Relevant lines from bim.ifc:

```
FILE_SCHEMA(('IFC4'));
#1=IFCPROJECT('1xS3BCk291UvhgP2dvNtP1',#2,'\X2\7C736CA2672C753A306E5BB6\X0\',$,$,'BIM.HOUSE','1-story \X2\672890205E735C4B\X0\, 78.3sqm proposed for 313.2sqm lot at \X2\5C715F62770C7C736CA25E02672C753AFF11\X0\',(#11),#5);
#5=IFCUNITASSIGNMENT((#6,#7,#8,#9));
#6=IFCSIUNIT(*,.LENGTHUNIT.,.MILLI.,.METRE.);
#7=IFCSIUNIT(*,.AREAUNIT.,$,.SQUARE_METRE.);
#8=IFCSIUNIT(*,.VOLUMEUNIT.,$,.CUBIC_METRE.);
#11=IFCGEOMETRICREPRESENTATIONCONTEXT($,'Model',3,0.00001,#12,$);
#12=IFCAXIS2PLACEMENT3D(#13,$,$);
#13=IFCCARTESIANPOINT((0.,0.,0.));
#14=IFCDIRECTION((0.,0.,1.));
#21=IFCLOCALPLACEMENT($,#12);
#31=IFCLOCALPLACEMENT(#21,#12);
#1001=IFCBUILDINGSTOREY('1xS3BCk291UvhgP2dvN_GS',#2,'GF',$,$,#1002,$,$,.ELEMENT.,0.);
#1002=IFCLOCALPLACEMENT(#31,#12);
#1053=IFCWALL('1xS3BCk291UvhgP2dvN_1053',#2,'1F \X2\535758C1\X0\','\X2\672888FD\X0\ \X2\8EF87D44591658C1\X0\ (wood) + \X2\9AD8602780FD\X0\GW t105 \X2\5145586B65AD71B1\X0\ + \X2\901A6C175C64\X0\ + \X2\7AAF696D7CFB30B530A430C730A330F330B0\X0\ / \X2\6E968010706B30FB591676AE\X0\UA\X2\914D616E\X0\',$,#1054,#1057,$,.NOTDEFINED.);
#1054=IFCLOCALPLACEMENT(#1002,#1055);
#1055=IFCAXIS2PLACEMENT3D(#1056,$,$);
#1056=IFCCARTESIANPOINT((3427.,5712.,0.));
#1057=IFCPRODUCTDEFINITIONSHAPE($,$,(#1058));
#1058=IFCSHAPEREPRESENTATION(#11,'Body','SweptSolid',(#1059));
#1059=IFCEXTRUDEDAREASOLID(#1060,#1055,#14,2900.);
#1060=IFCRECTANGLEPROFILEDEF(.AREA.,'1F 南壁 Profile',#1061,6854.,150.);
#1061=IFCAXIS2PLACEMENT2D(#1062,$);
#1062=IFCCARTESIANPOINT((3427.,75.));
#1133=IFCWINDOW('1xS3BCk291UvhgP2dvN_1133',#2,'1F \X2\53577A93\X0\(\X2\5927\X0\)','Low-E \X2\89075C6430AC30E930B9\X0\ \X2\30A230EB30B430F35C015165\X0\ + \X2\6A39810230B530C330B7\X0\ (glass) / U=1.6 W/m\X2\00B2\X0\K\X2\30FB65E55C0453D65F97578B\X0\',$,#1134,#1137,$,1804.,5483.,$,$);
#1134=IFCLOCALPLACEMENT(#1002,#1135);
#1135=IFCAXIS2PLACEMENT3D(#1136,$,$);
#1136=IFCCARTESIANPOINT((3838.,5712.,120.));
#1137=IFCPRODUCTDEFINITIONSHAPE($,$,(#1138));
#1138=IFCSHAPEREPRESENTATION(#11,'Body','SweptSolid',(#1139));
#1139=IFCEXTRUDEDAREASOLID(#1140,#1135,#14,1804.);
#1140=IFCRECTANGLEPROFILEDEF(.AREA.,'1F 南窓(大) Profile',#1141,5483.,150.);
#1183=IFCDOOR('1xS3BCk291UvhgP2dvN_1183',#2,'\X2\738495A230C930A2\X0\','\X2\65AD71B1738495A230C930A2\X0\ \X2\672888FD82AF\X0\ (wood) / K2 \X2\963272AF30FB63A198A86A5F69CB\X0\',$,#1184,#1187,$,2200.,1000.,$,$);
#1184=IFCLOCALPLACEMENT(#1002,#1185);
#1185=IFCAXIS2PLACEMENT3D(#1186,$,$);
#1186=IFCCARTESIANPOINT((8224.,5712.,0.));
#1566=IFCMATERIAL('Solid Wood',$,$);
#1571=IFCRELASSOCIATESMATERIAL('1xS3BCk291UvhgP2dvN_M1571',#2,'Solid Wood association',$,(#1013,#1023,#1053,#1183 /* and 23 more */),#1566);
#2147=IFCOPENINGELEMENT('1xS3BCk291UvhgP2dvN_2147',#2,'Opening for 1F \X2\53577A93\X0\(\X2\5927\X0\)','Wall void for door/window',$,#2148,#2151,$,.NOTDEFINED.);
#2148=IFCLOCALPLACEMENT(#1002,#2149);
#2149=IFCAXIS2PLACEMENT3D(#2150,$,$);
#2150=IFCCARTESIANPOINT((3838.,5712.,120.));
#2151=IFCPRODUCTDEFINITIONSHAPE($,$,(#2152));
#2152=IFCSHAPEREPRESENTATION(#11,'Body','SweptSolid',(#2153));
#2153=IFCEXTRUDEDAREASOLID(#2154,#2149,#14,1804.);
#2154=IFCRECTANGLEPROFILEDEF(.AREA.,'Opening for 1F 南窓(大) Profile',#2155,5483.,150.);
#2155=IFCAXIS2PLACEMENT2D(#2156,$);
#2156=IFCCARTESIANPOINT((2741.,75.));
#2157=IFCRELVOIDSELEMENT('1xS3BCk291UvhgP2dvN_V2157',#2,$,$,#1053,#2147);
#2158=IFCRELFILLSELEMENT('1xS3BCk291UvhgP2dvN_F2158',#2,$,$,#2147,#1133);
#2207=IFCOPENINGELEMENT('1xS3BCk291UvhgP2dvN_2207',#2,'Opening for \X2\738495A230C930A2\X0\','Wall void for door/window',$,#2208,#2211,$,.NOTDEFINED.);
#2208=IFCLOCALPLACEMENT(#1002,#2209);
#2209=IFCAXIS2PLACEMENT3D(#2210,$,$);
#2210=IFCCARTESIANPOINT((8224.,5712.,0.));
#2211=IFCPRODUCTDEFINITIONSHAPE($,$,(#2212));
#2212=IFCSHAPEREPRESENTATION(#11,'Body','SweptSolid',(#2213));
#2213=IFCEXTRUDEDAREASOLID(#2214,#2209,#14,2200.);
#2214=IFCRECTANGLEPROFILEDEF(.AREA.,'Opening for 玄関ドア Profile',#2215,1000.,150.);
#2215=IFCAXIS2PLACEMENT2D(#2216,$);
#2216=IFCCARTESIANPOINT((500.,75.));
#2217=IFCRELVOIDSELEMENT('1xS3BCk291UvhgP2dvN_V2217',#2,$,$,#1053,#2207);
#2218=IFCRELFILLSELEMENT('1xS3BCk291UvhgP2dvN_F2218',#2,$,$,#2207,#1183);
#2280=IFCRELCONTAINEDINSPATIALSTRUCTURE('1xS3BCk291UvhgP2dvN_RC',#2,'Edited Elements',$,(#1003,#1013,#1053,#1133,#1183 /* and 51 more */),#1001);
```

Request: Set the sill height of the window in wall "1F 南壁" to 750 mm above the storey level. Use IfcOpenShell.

```python
import numpy as np
import ifcopenshell
import ifcopenshell.api.geometry
import ifcopenshell.geom
import ifcopenshell.util.element
import ifcopenshell.util.placement
import ifcopenshell.util.shape
import ifcopenshell.util.unit

model = ifcopenshell.open("bim.ifc")
unit_scale = ifcopenshell.util.unit.calculate_unit_scale(model)

window = model.by_guid("1xS3BCk291UvhgP2dvN_1133")
opening = window.FillsVoids[0].RelatingOpeningElement
storey = ifcopenshell.util.element.get_container(window, ifc_class="IfcBuildingStorey")
level = ifcopenshell.util.placement.get_local_placement(storey.ObjectPlacement)[2, 3]

# The opening's origin need not be at the sill, so measure its lowest point.
shape = ifcopenshell.geom.create_shape(ifcopenshell.geom.settings(), opening)
bottom = ifcopenshell.util.shape.get_shape_bottom_elevation(shape, shape.geometry) / unit_scale
dz = level + 0.75 / unit_scale - bottom

shift = np.array([0.0, 0.0, dz])
# The window is not placed relative to its opening, so move both.
for product in (opening, window):
    matrix = ifcopenshell.util.placement.get_local_placement(product.ObjectPlacement)
    matrix[:3, 3] += shift
    ifcopenshell.api.geometry.edit_object_placement(model, product=product, matrix=matrix, is_si=False)

print(f"moved by {dz * unit_scale:+.3f} m")

model.write("bim_rev.ifc")
```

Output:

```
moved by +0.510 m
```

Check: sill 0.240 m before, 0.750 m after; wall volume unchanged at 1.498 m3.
